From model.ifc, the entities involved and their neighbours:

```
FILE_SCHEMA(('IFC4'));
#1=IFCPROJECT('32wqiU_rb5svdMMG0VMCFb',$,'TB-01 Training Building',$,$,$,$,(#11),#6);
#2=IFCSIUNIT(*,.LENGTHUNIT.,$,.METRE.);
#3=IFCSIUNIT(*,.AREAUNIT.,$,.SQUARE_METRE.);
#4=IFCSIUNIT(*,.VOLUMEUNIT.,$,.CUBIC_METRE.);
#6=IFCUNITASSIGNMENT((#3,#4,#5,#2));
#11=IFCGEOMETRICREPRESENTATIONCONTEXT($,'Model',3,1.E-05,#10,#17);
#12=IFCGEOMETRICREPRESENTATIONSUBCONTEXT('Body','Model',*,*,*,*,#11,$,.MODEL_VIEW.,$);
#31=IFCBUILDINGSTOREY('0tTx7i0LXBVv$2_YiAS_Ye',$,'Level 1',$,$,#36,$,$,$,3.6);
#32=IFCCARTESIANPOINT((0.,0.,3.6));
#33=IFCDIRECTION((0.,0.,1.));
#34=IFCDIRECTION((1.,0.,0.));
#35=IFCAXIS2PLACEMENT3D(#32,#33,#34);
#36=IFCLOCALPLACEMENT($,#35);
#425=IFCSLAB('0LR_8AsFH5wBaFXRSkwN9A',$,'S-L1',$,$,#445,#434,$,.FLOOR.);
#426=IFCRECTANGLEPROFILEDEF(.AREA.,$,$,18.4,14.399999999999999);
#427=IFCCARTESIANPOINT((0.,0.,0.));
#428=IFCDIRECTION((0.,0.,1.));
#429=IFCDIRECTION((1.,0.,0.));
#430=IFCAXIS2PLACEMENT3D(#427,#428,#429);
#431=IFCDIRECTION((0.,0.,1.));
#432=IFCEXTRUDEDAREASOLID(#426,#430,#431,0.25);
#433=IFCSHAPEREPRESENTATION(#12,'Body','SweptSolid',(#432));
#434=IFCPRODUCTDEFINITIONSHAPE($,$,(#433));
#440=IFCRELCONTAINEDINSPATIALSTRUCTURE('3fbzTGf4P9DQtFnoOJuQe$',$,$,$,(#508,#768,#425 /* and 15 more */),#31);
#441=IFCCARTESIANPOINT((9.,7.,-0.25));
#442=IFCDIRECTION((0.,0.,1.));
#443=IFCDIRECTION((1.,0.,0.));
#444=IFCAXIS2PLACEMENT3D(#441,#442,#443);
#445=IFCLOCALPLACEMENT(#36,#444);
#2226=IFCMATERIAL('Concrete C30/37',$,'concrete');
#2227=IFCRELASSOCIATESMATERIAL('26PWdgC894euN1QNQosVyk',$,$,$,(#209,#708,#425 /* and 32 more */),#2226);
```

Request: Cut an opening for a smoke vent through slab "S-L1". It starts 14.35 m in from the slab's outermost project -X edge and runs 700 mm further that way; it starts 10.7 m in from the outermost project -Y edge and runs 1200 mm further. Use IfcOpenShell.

```python
import numpy as np
import ifcopenshell
import ifcopenshell.api.feature
import ifcopenshell.api.geometry
import ifcopenshell.api.root
import ifcopenshell.geom
import ifcopenshell.util.placement
import ifcopenshell.util.representation
import ifcopenshell.util.shape
import ifcopenshell.util.unit

model = ifcopenshell.open("model.ifc")
unit_scale = ifcopenshell.util.unit.calculate_unit_scale(model)
settings = ifcopenshell.geom.settings()


def volume(element):
    """Net volume in cubic metres, openings subtracted."""
    shape = ifcopenshell.geom.create_shape(settings, element)
    return ifcopenshell.util.shape.get_volume(shape.geometry)


slab = model.by_guid("0LR_8AsFH5wBaFXRSkwN9A")
before = volume(slab)

# Extent in the slab's own axes, in metres. The edges named are its -X and -Y sides.
slab_shape = ifcopenshell.geom.create_shape(settings, slab)
vertices = ifcopenshell.util.shape.get_vertices(slab_shape.geometry)
x_min, y_min, bottom = vertices.min(axis=0)
top = vertices[:, 2].max()

opening = ifcopenshell.api.root.create_entity(model, ifc_class="IfcOpeningElement", name="Smoke vent opening", predefined_type="OPENING")
context = ifcopenshell.util.representation.get_context(model, "Model", "Body", "MODEL_VIEW")
width, depth = 0.7, 1.2
outline = [(0.0, 0.0), (width, 0.0), (width, depth), (0.0, depth), (0.0, 0.0)]
# Overshoot both faces by 50 mm so the cut is clean.
shape = ifcopenshell.api.geometry.add_slab_representation(
    model, context=context, depth=top - bottom + 0.1, polyline=outline
)
ifcopenshell.api.geometry.assign_representation(model, product=opening, representation=shape)

matrix = ifcopenshell.util.placement.get_local_placement(slab.ObjectPlacement)
matrix[:, 3] = matrix @ np.append(np.array([x_min + 14.35, y_min + 10.7, bottom - 0.05]) / unit_scale, 1.0)
ifcopenshell.api.geometry.edit_object_placement(model, product=opening, matrix=matrix, is_si=False)
ifcopenshell.api.feature.add_feature(model, feature=opening, element=slab)

after = volume(slab)

print(f"slab volume {before:.3f} -> {after:.3f} m3")

model.write("model-out.ifc")
```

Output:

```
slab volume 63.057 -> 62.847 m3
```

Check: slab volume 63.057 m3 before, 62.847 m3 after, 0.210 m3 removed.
